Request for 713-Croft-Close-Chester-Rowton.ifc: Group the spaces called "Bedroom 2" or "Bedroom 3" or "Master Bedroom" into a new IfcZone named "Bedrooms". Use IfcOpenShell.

First a look at what the model holds.

```python
import ifcopenshell

model = ifcopenshell.open("713-Croft-Close-Chester-Rowton.ifc")
print(model.schema)
seen = {}
for space in model.by_type("IfcSpace"):
    seen[space.LongName] = seen.get(space.LongName, 0) + 1
for name, count in sorted(seen.items(), key=str):
    print(count, "x", name)
print("zones:", [z.Name for z in model.by_type("IfcZone")][:20])
```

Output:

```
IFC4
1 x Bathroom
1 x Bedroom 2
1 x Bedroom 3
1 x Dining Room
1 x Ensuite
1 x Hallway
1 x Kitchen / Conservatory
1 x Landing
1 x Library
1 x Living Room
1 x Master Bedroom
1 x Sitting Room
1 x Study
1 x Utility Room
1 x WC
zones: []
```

```python
import ifcopenshell
import ifcopenshell.api.group
import ifcopenshell.api.root

model = ifcopenshell.open("713-Croft-Close-Chester-Rowton.ifc")

names = {"Bedroom 2", "Bedroom 3", "Master Bedroom"}
spaces = [s for s in model.by_type("IfcSpace") if s.LongName in names]

zone = ifcopenshell.api.root.create_entity(model, ifc_class="IfcZone", name="Bedrooms")
ifcopenshell.api.group.assign_group(model, products=spaces, group=zone)
print(len(spaces), "spaces in", zone.Name)

model.write("713-Croft-Close-Chester-Rowton_v2.ifc")
```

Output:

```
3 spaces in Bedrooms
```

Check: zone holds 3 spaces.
